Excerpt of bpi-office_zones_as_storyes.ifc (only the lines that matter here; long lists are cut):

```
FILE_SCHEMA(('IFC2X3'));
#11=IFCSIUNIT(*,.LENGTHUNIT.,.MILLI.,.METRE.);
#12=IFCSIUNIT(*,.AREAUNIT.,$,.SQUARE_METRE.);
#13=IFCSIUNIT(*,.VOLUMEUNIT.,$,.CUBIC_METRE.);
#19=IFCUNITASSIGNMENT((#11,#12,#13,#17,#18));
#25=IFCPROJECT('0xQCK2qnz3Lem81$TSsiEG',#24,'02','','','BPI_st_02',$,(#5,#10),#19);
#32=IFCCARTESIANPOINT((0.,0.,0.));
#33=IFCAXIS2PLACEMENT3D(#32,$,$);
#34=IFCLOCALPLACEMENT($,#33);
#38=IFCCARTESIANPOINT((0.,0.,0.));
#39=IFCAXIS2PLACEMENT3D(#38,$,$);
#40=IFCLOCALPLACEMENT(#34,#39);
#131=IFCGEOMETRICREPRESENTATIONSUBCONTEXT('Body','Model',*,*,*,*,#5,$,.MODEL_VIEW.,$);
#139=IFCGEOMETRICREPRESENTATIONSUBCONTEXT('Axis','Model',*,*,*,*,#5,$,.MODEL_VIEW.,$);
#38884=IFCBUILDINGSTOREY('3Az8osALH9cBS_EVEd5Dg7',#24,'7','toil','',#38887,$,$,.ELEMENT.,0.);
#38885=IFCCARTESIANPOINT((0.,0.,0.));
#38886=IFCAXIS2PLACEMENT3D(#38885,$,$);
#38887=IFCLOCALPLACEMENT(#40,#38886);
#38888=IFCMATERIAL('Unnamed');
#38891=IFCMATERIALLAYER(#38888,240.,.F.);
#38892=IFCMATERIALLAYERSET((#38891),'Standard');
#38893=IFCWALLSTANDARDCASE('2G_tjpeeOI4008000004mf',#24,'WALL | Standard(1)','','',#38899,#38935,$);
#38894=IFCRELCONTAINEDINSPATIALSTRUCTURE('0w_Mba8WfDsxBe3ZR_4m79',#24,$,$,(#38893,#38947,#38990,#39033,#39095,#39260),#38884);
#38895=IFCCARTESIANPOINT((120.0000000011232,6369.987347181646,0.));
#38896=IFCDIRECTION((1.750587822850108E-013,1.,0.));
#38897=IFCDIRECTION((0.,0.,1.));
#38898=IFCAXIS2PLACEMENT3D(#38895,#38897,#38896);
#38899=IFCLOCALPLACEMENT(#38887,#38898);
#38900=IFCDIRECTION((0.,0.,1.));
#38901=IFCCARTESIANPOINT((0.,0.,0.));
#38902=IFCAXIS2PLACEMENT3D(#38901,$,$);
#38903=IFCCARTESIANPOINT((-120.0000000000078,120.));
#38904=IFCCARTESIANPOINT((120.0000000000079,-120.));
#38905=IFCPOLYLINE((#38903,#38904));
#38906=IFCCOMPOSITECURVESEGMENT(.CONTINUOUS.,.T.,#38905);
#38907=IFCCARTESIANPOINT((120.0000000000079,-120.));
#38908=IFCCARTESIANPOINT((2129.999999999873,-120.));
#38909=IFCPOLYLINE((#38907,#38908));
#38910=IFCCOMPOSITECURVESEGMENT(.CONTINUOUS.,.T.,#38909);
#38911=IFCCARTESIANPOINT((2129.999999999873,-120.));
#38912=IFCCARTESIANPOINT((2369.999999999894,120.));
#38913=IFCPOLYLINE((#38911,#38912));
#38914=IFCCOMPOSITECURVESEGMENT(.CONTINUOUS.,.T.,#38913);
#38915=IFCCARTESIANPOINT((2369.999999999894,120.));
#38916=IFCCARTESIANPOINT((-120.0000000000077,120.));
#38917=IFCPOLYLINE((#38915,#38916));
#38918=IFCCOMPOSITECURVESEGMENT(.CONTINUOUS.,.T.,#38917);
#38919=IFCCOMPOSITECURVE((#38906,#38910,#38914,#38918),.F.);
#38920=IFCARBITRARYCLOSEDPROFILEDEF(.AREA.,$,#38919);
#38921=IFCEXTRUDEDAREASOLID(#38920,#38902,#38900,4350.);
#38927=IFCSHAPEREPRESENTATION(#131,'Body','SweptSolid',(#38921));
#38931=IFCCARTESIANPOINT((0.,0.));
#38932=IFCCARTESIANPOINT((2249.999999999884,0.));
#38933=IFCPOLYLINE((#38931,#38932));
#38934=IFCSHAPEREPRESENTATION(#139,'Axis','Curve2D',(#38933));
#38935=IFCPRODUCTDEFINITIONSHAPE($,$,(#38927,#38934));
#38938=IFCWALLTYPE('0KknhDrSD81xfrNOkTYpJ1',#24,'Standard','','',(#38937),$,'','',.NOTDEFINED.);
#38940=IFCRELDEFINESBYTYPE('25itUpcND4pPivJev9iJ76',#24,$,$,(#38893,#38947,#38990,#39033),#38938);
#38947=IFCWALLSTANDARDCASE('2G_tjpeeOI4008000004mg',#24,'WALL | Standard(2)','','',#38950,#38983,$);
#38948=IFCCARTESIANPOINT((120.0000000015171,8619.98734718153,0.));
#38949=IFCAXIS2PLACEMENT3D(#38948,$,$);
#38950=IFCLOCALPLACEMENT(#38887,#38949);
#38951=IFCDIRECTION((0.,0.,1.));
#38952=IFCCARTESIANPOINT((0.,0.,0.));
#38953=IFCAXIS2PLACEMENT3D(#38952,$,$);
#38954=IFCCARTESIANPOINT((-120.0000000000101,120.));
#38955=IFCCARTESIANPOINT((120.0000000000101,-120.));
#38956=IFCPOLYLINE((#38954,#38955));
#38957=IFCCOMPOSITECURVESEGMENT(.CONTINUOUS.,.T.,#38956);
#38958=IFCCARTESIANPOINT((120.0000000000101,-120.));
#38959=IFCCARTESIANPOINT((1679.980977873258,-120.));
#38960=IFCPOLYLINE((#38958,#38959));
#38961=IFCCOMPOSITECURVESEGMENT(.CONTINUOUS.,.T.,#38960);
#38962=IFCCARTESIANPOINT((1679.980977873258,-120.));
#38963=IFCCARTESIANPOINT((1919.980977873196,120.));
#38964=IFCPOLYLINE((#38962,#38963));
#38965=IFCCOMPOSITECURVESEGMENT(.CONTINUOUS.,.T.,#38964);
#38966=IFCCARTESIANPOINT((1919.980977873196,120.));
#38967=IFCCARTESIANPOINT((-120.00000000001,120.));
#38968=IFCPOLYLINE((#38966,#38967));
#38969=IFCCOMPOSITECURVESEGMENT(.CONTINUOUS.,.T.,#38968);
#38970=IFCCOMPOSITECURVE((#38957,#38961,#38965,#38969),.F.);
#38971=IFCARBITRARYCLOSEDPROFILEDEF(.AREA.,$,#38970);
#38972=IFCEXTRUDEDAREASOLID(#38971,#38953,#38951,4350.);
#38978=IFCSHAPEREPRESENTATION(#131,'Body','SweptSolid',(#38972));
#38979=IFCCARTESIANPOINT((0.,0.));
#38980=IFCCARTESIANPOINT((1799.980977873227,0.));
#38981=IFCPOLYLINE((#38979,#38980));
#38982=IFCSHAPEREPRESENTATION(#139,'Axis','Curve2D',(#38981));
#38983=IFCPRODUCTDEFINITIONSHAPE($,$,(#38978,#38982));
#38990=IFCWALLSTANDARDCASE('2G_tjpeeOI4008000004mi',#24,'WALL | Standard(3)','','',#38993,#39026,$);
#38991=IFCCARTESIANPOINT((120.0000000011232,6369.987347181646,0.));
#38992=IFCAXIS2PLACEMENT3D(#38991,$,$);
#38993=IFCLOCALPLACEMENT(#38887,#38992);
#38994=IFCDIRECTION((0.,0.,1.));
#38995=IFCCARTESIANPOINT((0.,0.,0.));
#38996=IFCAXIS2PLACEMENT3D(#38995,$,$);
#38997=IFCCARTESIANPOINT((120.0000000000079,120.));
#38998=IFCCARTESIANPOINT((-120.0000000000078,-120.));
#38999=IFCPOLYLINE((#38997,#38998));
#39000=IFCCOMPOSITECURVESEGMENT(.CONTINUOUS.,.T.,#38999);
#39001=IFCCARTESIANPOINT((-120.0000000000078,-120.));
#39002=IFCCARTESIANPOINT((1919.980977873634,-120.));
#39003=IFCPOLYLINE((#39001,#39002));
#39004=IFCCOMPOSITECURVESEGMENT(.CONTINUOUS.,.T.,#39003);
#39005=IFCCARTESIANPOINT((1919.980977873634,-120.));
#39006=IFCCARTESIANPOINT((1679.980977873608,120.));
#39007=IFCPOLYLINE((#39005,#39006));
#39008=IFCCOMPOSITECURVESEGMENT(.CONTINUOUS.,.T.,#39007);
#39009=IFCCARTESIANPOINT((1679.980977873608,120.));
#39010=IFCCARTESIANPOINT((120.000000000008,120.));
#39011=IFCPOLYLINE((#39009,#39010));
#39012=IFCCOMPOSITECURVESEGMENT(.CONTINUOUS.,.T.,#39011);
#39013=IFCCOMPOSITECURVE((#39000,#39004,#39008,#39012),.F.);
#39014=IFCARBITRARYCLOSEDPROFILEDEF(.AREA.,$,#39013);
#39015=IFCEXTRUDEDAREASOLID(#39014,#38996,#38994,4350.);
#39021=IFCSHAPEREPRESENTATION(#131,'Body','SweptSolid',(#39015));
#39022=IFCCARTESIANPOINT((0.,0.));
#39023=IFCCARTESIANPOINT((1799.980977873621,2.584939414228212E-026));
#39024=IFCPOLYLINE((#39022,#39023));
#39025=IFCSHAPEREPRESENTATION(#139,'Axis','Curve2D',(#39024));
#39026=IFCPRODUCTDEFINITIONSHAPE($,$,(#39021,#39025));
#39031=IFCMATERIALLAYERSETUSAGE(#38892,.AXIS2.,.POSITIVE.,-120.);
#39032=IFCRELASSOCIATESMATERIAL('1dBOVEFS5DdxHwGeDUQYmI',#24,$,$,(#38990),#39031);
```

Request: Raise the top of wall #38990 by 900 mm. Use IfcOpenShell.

```python
import ifcopenshell
import ifcopenshell.geom
import ifcopenshell.util.representation
import ifcopenshell.util.shape
import ifcopenshell.util.unit

model = ifcopenshell.open("bpi-office_zones_as_storyes.ifc")
unit_scale = ifcopenshell.util.unit.calculate_unit_scale(model)
settings = ifcopenshell.geom.settings()


def volume(element):
    """Net volume in cubic metres, openings subtracted."""
    shape = ifcopenshell.geom.create_shape(settings, element)
    return ifcopenshell.util.shape.get_volume(shape.geometry)


wall = model.by_guid("2G_tjpeeOI4008000004mi")
before = volume(wall)

body = ifcopenshell.util.representation.get_representation(wall, "Model", "Body")
solid = body.Items[0]
old_height = solid.Depth
solid.Depth += 0.9 / unit_scale
after = volume(wall)

print(f"height {old_height:g} -> {solid.Depth:g}, volume {before:.3f} -> {after:.3f} m3")

model.write("bpi-office_zones_as_storyes_v2.ifc")
```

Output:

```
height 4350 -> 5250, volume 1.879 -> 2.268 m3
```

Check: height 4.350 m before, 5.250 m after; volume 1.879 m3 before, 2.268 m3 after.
